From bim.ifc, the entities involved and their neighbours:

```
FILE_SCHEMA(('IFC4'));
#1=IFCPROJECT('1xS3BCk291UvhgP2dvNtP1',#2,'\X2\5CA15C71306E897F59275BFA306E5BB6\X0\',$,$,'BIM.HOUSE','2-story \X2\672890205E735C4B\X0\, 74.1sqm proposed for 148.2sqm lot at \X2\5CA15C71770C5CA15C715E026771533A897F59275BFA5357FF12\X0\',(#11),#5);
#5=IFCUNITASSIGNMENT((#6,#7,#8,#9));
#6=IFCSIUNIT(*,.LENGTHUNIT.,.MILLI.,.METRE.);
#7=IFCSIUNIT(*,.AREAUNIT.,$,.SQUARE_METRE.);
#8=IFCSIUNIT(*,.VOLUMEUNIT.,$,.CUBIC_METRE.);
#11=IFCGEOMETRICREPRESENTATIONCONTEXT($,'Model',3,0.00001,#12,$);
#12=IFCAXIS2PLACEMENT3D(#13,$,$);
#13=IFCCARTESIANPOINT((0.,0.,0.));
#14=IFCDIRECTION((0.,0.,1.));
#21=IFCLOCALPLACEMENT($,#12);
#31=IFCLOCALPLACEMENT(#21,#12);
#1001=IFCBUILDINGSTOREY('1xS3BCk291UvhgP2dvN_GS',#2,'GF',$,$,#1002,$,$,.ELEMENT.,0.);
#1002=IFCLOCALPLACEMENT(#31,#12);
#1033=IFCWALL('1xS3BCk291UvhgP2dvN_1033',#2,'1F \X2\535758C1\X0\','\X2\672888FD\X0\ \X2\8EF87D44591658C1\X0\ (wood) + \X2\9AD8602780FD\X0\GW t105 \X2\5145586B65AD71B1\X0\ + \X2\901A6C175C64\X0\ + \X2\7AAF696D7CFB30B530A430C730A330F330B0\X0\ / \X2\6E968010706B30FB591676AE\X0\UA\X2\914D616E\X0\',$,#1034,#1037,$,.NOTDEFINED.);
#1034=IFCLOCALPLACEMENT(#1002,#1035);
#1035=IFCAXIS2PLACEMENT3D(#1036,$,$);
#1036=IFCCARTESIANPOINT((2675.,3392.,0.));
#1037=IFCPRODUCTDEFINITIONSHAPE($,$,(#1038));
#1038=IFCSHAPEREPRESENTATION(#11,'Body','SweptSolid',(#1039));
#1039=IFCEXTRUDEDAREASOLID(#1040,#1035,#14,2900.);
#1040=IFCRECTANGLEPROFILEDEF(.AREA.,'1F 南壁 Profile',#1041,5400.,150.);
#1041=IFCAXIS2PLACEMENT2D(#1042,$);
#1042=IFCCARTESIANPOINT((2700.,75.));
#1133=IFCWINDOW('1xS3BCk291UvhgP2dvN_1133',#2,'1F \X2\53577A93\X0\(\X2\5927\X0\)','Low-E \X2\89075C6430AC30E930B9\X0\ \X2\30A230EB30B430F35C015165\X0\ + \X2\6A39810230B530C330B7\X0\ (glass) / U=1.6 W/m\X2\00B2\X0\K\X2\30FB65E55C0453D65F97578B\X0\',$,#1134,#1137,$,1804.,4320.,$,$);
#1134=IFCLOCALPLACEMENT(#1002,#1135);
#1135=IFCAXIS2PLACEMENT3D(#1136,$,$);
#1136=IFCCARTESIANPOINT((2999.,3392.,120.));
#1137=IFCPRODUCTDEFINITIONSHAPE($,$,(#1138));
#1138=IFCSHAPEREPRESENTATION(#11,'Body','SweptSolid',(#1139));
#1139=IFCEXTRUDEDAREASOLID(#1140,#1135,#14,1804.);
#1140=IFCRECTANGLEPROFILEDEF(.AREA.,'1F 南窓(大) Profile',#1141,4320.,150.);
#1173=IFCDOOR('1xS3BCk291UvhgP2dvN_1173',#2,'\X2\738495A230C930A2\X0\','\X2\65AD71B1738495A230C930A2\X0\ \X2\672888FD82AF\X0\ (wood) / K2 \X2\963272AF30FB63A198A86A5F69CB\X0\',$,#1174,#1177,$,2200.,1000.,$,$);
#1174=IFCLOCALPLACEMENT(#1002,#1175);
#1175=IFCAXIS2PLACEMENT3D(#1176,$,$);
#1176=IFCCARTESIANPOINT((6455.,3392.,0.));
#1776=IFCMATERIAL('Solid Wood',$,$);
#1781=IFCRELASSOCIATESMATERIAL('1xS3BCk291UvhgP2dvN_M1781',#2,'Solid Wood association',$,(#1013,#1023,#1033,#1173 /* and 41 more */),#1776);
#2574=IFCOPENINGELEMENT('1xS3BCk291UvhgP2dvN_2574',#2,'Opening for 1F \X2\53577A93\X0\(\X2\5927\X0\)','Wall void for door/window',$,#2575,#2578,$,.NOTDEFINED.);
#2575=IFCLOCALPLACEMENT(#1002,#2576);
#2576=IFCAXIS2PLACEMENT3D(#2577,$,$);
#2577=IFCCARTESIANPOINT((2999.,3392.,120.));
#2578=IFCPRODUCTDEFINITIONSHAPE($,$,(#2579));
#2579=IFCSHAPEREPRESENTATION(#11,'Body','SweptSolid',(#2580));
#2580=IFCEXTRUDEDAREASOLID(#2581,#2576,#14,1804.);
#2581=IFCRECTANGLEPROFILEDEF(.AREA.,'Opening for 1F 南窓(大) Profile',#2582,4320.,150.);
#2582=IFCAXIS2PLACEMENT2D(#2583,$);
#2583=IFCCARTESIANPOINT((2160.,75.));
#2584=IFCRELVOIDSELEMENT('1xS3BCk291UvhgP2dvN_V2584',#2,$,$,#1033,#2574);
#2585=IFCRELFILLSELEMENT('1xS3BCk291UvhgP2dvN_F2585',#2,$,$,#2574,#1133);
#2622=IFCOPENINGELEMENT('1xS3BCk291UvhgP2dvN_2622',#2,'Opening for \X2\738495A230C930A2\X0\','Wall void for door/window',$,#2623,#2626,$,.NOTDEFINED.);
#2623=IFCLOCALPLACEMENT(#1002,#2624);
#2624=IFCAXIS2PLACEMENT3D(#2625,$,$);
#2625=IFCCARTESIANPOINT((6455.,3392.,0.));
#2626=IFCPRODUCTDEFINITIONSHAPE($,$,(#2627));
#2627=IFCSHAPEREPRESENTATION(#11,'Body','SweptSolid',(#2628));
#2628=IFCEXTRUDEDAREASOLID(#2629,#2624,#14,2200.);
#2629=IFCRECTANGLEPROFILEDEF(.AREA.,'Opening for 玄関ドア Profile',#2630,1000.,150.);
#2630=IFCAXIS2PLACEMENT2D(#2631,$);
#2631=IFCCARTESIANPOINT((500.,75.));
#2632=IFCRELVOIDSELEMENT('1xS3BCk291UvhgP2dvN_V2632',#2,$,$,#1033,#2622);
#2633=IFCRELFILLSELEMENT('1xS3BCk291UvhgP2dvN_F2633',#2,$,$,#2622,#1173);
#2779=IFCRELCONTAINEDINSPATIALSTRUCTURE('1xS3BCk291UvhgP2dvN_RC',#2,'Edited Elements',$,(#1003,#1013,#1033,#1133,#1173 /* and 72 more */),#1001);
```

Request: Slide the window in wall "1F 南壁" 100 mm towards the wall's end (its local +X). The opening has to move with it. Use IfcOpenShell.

```python
import ifcopenshell
import ifcopenshell.api.geometry
import ifcopenshell.util.placement

model = ifcopenshell.open("bim.ifc")

window = model.by_id(1133)
opening = window.FillsVoids[0].RelatingOpeningElement
wall = opening.VoidsElements[0].RelatingBuildingElement

wall_matrix = ifcopenshell.util.placement.get_local_placement(wall.ObjectPlacement)
shift = wall_matrix[:3, 0] * 100.0
before = ifcopenshell.util.placement.get_local_placement(window.ObjectPlacement)[:3, 3].copy()

# The window is not placed relative to its opening, so move both.
for product in (opening, window):
    matrix = ifcopenshell.util.placement.get_local_placement(product.ObjectPlacement)
    matrix[:3, 3] += shift
    ifcopenshell.api.geometry.edit_object_placement(model, product=product, matrix=matrix, is_si=False)

after = ifcopenshell.util.placement.get_local_placement(window.ObjectPlacement)[:3, 3]
print("window moved by", (after - before).round(3) + 0.0)

model.write("bim-out.ifc")
```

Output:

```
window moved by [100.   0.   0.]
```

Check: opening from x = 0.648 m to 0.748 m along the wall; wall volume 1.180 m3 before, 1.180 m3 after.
